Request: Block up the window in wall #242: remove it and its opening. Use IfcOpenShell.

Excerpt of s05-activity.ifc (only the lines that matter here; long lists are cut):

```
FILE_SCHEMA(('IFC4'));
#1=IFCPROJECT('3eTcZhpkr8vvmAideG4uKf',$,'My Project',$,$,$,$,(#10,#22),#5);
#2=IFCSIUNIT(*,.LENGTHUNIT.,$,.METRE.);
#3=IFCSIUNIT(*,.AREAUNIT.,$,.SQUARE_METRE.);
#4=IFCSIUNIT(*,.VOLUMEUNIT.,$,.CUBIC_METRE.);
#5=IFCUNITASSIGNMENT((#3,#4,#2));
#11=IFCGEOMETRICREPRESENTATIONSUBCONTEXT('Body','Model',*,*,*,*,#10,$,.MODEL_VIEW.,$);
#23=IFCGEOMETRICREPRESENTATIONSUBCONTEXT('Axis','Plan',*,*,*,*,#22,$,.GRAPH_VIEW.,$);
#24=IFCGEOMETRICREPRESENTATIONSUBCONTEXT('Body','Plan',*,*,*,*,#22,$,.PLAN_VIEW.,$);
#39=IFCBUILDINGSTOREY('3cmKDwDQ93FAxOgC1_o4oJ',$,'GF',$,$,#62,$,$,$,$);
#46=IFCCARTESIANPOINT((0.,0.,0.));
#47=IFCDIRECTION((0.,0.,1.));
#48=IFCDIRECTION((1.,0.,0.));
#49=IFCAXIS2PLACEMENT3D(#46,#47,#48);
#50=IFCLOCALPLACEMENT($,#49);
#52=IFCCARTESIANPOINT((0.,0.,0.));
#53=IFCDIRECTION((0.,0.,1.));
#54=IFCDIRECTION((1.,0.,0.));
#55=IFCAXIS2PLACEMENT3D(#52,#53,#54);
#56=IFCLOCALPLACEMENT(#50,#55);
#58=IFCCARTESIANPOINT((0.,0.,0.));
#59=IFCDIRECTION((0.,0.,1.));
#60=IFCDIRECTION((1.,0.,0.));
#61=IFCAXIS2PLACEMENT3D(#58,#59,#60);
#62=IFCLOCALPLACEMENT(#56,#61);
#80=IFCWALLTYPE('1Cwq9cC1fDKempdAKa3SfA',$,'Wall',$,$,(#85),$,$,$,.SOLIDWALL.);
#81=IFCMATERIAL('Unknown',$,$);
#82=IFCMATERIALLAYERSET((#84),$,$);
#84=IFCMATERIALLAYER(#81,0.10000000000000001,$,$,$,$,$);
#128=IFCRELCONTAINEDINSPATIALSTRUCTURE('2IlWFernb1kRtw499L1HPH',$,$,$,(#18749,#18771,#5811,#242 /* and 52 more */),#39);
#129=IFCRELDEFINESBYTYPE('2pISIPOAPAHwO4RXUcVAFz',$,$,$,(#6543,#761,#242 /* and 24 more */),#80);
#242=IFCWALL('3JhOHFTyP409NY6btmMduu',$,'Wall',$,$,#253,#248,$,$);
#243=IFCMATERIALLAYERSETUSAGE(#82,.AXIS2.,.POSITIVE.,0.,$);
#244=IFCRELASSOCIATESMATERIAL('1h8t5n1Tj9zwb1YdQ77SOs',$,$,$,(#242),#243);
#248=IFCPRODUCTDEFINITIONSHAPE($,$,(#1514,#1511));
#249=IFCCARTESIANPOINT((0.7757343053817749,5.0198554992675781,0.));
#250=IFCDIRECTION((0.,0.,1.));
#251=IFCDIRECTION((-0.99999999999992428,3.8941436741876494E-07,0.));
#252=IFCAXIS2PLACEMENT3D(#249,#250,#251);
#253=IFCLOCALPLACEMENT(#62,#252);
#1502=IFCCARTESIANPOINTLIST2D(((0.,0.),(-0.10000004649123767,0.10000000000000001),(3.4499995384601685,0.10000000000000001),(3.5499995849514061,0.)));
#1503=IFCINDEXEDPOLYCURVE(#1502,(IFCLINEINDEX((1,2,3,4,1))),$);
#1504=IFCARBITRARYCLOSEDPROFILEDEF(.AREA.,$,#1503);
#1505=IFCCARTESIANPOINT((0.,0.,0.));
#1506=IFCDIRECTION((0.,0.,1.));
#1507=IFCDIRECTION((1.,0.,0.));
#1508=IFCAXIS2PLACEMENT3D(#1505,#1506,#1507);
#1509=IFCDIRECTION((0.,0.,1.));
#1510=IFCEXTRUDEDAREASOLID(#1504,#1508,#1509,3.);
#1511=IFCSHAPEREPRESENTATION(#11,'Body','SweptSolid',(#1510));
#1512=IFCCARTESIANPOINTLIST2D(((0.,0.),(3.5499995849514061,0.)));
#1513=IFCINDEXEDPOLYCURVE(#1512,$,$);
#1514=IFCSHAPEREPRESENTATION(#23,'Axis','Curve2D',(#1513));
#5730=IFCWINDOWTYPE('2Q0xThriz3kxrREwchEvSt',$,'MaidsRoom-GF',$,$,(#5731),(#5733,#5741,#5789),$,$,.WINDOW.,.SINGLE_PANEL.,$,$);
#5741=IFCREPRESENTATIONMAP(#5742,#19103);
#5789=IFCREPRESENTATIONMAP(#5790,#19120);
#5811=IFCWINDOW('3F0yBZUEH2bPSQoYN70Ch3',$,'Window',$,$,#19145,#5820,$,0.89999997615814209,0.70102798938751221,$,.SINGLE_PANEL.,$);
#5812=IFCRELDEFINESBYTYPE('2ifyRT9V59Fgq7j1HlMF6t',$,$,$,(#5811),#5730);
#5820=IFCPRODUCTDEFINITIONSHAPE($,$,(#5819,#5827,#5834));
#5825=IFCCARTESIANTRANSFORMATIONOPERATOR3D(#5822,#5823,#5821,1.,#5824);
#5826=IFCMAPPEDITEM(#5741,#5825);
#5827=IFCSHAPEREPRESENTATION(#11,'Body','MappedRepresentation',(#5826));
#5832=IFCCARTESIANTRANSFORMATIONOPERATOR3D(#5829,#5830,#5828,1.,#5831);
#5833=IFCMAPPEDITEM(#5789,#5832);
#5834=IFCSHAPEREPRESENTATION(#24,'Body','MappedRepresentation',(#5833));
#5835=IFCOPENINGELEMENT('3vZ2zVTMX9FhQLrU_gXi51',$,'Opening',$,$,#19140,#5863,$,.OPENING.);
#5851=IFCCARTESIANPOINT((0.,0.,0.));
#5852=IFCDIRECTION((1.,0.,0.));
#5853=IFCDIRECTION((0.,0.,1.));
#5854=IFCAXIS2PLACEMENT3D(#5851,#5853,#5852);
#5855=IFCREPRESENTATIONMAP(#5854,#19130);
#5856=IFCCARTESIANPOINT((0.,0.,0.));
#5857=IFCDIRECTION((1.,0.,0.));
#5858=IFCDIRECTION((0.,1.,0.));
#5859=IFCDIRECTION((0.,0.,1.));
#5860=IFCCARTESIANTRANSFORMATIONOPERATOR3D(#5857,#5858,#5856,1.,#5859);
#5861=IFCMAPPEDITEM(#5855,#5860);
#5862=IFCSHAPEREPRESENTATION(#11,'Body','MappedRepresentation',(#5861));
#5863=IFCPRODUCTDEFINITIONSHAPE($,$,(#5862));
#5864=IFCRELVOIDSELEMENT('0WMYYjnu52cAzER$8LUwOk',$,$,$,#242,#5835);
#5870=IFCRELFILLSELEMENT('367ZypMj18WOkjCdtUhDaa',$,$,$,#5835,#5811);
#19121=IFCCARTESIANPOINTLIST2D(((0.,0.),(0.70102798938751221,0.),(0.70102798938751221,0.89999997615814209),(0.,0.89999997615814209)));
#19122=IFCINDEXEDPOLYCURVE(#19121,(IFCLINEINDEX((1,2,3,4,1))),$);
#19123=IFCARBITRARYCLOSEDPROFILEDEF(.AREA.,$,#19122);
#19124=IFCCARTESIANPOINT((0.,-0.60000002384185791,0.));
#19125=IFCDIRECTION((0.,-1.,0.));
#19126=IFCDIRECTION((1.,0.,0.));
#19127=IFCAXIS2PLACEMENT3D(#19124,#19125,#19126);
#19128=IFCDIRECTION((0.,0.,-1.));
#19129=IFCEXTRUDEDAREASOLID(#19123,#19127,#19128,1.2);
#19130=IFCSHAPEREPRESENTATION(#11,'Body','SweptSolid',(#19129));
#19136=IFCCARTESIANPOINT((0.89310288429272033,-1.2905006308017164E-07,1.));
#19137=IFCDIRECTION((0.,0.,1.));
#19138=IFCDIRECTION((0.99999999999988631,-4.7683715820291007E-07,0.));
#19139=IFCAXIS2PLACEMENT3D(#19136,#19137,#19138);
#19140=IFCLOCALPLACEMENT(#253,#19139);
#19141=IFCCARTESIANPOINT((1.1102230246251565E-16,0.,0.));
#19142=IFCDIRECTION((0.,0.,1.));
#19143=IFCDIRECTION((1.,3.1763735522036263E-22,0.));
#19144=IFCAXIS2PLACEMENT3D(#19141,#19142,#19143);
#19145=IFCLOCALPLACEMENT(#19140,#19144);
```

```python
import ifcopenshell
import ifcopenshell.api.feature
import ifcopenshell.api.root
import ifcopenshell.geom
import ifcopenshell.util.shape

model = ifcopenshell.open("s05-activity.ifc")
settings = ifcopenshell.geom.settings()


def volume(element):
    """Net volume in cubic metres, openings subtracted."""
    shape = ifcopenshell.geom.create_shape(settings, element)
    return ifcopenshell.util.shape.get_volume(shape.geometry)


window = model.by_guid("3F0yBZUEH2bPSQoYN70Ch3")
opening = window.FillsVoids[0].RelatingOpeningElement
wall = opening.VoidsElements[0].RelatingBuildingElement
before = volume(wall)

ifcopenshell.api.root.remove_product(model, product=window)
ifcopenshell.api.feature.remove_feature(model, feature=opening)

after = volume(wall)

print(f"wall volume {before:.3f} -> {after:.3f} m3")

model.write("s05-activity_updated.ifc")
```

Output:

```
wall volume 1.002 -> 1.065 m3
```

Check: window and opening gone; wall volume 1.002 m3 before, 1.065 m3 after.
